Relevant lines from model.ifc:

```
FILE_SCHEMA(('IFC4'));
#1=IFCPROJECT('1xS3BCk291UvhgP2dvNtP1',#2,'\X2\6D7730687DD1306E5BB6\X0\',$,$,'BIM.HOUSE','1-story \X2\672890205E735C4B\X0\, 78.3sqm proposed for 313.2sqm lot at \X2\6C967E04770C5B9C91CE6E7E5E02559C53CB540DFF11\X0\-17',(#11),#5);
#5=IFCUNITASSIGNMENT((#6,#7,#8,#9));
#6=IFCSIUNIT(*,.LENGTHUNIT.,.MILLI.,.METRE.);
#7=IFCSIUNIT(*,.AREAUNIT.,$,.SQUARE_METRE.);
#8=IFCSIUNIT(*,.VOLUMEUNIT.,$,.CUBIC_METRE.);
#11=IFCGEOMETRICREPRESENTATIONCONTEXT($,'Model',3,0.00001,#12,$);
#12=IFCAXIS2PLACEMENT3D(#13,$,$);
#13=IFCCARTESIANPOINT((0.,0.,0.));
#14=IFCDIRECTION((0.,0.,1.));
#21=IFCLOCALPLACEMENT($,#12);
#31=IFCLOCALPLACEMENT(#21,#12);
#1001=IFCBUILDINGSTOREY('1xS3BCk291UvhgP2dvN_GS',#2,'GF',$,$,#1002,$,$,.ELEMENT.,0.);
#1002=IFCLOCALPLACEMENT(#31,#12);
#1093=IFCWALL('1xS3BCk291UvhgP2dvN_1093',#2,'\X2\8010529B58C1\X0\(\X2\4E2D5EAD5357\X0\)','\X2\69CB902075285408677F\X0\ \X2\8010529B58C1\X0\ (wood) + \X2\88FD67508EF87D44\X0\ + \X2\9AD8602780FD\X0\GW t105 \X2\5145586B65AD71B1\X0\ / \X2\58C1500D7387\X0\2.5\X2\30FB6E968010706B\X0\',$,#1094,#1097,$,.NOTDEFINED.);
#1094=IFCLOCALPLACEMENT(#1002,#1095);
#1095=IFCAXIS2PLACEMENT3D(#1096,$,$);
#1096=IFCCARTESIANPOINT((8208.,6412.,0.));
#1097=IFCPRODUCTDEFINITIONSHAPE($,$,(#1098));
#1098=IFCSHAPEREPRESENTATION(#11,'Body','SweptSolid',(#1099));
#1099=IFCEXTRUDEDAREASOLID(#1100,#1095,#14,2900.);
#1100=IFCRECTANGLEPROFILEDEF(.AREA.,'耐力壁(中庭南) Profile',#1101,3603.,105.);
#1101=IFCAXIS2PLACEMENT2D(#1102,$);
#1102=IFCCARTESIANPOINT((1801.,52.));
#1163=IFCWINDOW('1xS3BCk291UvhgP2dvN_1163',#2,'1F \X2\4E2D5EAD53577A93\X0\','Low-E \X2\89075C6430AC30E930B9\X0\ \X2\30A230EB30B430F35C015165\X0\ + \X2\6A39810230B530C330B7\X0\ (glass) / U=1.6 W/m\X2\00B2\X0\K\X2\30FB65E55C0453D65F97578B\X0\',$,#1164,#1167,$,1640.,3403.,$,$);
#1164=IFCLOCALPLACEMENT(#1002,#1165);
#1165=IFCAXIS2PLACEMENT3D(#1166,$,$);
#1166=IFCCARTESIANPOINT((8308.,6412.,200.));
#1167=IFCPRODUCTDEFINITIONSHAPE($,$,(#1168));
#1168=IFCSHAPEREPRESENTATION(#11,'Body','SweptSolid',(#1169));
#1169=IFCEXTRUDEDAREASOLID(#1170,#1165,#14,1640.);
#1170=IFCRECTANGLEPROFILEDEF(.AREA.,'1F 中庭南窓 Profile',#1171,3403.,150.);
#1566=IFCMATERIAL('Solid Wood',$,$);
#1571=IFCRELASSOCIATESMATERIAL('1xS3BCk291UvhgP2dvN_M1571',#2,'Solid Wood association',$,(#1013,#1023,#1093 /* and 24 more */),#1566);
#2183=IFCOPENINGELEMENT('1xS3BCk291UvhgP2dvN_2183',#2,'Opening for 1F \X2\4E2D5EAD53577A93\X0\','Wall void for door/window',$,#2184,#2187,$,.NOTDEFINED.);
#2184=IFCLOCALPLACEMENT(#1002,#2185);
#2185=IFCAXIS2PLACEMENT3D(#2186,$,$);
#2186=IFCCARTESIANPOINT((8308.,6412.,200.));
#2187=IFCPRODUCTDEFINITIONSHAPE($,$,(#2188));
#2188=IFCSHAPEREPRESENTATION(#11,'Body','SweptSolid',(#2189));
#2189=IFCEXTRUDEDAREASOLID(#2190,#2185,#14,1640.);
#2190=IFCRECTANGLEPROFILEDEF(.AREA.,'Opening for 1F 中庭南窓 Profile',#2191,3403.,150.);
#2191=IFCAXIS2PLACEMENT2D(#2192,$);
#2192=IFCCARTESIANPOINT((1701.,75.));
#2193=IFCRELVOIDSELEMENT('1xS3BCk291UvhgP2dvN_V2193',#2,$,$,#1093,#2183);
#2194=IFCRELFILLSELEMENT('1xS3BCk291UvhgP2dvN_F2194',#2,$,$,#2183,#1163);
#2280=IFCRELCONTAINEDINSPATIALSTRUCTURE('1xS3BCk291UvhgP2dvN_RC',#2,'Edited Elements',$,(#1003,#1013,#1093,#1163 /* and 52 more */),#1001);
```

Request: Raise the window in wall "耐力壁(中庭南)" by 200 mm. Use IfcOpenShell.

```python
import numpy as np
import ifcopenshell
import ifcopenshell.api.geometry
import ifcopenshell.util.placement
import ifcopenshell.util.unit

model = ifcopenshell.open("model.ifc")
unit_scale = ifcopenshell.util.unit.calculate_unit_scale(model)

window = model.by_id(1163)
opening = window.FillsVoids[0].RelatingOpeningElement
dz = 200.0

shift = np.array([0.0, 0.0, dz])
# The window is not placed relative to its opening, so move both.
for product in (opening, window):
    matrix = ifcopenshell.util.placement.get_local_placement(product.ObjectPlacement)
    matrix[:3, 3] += shift
    ifcopenshell.api.geometry.edit_object_placement(model, product=product, matrix=matrix, is_si=False)

print(f"moved by {dz * unit_scale:+.3f} m")

model.write("model_edited.ifc")
```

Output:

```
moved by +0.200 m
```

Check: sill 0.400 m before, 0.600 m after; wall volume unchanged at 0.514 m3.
